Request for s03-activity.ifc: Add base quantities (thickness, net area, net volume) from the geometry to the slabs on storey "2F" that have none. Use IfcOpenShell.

First a look at what the model holds.

```python
import ifcopenshell
import ifcopenshell.util.element
import ifcopenshell.util.unit

model = ifcopenshell.open("s03-activity.ifc")
print(model.schema)
for unit_type in ("LENGTHUNIT", "AREAUNIT", "VOLUMEUNIT"):
    print(unit_type, ifcopenshell.util.unit.calculate_unit_scale(model, unit_type))
storey = next(s for s in model.by_type("IfcBuildingStorey") if s.Name == "2F")
slabs = [e for e in ifcopenshell.util.element.get_decomposition(storey) if e.is_a("IfcSlab")]
for e in sorted(slabs, key=lambda e: e.id()):
    print(e.id(), e.is_a(), e.Name, list(ifcopenshell.util.element.get_psets(e, qtos_only=True)), sep=" | ")
```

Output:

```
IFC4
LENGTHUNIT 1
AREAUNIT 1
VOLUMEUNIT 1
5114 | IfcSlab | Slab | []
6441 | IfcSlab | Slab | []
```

```python
import ifcopenshell
import ifcopenshell.api.pset
import ifcopenshell.geom
import ifcopenshell.util.element
import ifcopenshell.util.shape
import ifcopenshell.util.unit

model = ifcopenshell.open("s03-activity.ifc")
unit_scale = ifcopenshell.util.unit.calculate_unit_scale(model)
area_scale = ifcopenshell.util.unit.calculate_unit_scale(model, "AREAUNIT")
volume_scale = ifcopenshell.util.unit.calculate_unit_scale(model, "VOLUMEUNIT")
settings = ifcopenshell.geom.settings()

storey = next(s for s in model.by_type("IfcBuildingStorey") if s.Name == "2F")
slabs = [e for e in ifcopenshell.util.element.get_decomposition(storey) if e.is_a("IfcSlab")]

for e in sorted(slabs, key=lambda e: e.id()):
    if ifcopenshell.util.element.get_psets(e, qtos_only=True, should_inherit=False):
        continue
    # Geometry comes back in metres, in the element's own axes.
    shape = ifcopenshell.geom.create_shape(settings, e)
    values = {
        "Width": ifcopenshell.util.shape.get_z(shape.geometry) / unit_scale,
        "NetArea": ifcopenshell.util.shape.get_footprint_area(shape.geometry) / area_scale,
        "NetVolume": ifcopenshell.util.shape.get_volume(shape.geometry) / volume_scale,
    }
    qto = ifcopenshell.api.pset.add_qto(model, product=e, name="Qto_SlabBaseQuantities")
    ifcopenshell.api.pset.edit_qto(model, qto=qto, properties=values)
    print(e.id(), {k: round(v, 3) for k, v in values.items()})

model.write("s03-activity_v2.ifc")
```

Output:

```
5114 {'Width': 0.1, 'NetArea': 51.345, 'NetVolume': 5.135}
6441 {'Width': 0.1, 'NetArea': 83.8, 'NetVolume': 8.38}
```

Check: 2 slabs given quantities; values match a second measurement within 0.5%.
